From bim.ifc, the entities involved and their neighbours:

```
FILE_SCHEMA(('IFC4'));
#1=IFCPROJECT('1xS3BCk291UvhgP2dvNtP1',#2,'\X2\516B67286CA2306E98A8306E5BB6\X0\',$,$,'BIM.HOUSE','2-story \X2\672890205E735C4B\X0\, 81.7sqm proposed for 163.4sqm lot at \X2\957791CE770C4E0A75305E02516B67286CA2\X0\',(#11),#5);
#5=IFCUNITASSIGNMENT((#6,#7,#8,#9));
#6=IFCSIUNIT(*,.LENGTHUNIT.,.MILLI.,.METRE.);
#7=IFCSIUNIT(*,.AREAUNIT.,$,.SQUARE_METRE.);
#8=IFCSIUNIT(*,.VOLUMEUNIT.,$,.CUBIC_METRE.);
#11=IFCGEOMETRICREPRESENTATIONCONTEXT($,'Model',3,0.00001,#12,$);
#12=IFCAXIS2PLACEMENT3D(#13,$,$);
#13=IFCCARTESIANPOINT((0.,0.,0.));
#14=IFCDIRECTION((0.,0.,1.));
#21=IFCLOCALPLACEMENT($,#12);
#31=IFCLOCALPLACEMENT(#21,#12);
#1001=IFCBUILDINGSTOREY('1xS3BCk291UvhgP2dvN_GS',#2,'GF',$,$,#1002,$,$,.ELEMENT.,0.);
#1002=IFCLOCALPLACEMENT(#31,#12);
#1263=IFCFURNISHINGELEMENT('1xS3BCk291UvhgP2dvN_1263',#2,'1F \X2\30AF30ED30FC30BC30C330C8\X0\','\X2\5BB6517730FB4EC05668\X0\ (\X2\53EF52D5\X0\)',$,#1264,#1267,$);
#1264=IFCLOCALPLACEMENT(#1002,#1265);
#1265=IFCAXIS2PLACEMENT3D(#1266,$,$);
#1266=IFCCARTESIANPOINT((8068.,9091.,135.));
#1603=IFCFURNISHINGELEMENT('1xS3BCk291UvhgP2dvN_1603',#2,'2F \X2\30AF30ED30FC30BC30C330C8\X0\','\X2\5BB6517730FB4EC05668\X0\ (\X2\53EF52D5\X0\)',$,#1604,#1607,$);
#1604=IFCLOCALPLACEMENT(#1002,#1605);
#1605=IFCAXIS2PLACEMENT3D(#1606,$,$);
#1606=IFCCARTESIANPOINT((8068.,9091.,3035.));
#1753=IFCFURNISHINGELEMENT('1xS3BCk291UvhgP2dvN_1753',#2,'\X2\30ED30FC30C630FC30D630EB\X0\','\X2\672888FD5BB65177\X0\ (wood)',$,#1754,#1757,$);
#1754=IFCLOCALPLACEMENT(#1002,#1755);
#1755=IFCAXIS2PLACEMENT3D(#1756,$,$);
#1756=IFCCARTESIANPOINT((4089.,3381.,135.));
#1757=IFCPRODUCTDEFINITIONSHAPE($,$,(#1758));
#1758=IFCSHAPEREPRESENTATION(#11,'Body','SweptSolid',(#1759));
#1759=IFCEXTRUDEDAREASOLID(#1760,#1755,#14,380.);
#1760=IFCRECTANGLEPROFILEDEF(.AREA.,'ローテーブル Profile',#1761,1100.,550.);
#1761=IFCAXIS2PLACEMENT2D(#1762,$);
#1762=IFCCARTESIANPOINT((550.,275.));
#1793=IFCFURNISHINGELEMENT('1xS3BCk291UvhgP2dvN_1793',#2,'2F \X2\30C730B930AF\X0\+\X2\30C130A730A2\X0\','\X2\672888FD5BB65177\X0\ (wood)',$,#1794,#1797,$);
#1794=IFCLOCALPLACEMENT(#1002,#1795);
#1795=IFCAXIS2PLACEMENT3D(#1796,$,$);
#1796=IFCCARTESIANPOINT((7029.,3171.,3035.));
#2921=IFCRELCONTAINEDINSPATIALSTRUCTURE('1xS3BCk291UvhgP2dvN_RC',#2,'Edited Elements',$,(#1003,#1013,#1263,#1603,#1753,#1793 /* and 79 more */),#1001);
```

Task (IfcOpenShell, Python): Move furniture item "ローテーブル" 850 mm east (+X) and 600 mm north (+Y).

```python
import ifcopenshell
import ifcopenshell.api.geometry
import ifcopenshell.util.placement
import ifcopenshell.util.unit

model = ifcopenshell.open("bim.ifc")
unit_scale = ifcopenshell.util.unit.calculate_unit_scale(model)

item = model.by_id(1753)
matrix = ifcopenshell.util.placement.get_local_placement(item.ObjectPlacement)
matrix[0, 3] += 0.85 / unit_scale
matrix[1, 3] += 0.6 / unit_scale
ifcopenshell.api.geometry.edit_object_placement(model, product=item, matrix=matrix, is_si=False)

print(ifcopenshell.util.placement.get_local_placement(item.ObjectPlacement).round(3) + 0.0)

model.write("bim-out.ifc")
```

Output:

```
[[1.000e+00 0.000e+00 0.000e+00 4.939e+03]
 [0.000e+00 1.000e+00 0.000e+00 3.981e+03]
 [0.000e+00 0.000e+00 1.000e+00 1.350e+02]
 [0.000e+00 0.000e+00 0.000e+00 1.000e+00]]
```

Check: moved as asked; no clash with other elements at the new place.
